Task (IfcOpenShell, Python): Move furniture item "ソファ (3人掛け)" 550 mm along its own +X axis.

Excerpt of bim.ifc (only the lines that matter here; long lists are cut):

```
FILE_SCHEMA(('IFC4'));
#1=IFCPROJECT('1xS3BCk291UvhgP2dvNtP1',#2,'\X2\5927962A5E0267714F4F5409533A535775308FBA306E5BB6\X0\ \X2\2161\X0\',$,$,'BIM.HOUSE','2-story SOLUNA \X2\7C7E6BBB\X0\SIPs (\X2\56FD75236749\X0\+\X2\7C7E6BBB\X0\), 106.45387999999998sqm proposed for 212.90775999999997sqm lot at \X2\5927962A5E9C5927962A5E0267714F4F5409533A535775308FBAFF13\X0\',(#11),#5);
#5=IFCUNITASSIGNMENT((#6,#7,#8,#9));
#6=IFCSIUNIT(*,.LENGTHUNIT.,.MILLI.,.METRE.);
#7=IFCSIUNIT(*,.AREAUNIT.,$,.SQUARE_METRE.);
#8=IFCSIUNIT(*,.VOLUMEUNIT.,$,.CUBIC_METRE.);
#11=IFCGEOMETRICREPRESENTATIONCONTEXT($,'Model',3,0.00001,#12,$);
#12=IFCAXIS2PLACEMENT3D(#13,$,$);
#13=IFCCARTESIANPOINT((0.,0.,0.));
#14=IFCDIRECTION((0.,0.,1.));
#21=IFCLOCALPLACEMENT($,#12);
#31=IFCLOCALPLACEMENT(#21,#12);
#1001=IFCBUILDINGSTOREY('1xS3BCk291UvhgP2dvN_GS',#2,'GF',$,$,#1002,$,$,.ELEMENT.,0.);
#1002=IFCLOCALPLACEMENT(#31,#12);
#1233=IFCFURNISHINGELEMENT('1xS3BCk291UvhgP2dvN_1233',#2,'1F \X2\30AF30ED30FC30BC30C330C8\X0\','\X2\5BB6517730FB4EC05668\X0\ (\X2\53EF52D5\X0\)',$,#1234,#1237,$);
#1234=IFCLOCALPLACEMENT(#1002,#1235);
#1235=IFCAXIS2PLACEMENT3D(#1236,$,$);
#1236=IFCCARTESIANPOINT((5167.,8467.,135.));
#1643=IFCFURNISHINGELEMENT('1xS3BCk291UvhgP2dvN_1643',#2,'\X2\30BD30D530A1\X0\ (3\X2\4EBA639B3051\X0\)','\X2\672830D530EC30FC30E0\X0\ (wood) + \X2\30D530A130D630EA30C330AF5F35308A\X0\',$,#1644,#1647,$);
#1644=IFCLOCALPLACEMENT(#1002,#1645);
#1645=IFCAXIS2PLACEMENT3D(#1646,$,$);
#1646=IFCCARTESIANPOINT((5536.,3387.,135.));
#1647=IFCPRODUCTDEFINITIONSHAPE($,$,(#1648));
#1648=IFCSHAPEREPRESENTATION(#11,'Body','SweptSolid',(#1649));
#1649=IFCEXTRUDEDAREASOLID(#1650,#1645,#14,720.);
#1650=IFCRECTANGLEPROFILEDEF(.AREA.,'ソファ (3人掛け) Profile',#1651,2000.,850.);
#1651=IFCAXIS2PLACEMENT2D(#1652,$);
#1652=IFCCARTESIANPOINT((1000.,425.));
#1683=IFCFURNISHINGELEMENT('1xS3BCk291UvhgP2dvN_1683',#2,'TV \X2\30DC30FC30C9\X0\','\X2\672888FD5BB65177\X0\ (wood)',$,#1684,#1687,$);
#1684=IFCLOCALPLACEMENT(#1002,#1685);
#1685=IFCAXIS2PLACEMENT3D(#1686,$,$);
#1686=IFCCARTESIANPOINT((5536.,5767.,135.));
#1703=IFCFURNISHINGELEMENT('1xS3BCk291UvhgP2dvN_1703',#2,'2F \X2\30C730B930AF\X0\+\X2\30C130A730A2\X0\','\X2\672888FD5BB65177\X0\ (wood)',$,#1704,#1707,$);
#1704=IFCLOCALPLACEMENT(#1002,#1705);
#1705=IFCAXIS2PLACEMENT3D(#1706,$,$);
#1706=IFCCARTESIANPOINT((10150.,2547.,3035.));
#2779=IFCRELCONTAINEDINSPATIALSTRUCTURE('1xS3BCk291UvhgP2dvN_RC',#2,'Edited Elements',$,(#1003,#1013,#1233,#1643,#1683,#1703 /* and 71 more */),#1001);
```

```python
import ifcopenshell
import ifcopenshell.api.geometry
import ifcopenshell.util.placement
import ifcopenshell.util.unit

model = ifcopenshell.open("bim.ifc")
unit_scale = ifcopenshell.util.unit.calculate_unit_scale(model)

item = model.by_guid("1xS3BCk291UvhgP2dvN_1643")
matrix = ifcopenshell.util.placement.get_local_placement(item.ObjectPlacement)
matrix[:3, 3] += matrix[:3, 0] * 0.55 / unit_scale
ifcopenshell.api.geometry.edit_object_placement(model, product=item, matrix=matrix, is_si=False)

print(ifcopenshell.util.placement.get_local_placement(item.ObjectPlacement).round(3) + 0.0)

model.write("bim_updated.ifc")
```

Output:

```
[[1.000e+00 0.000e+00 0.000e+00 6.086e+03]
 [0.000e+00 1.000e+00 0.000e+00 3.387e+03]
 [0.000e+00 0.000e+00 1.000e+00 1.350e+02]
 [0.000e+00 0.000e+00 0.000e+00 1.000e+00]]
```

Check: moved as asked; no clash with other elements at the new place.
